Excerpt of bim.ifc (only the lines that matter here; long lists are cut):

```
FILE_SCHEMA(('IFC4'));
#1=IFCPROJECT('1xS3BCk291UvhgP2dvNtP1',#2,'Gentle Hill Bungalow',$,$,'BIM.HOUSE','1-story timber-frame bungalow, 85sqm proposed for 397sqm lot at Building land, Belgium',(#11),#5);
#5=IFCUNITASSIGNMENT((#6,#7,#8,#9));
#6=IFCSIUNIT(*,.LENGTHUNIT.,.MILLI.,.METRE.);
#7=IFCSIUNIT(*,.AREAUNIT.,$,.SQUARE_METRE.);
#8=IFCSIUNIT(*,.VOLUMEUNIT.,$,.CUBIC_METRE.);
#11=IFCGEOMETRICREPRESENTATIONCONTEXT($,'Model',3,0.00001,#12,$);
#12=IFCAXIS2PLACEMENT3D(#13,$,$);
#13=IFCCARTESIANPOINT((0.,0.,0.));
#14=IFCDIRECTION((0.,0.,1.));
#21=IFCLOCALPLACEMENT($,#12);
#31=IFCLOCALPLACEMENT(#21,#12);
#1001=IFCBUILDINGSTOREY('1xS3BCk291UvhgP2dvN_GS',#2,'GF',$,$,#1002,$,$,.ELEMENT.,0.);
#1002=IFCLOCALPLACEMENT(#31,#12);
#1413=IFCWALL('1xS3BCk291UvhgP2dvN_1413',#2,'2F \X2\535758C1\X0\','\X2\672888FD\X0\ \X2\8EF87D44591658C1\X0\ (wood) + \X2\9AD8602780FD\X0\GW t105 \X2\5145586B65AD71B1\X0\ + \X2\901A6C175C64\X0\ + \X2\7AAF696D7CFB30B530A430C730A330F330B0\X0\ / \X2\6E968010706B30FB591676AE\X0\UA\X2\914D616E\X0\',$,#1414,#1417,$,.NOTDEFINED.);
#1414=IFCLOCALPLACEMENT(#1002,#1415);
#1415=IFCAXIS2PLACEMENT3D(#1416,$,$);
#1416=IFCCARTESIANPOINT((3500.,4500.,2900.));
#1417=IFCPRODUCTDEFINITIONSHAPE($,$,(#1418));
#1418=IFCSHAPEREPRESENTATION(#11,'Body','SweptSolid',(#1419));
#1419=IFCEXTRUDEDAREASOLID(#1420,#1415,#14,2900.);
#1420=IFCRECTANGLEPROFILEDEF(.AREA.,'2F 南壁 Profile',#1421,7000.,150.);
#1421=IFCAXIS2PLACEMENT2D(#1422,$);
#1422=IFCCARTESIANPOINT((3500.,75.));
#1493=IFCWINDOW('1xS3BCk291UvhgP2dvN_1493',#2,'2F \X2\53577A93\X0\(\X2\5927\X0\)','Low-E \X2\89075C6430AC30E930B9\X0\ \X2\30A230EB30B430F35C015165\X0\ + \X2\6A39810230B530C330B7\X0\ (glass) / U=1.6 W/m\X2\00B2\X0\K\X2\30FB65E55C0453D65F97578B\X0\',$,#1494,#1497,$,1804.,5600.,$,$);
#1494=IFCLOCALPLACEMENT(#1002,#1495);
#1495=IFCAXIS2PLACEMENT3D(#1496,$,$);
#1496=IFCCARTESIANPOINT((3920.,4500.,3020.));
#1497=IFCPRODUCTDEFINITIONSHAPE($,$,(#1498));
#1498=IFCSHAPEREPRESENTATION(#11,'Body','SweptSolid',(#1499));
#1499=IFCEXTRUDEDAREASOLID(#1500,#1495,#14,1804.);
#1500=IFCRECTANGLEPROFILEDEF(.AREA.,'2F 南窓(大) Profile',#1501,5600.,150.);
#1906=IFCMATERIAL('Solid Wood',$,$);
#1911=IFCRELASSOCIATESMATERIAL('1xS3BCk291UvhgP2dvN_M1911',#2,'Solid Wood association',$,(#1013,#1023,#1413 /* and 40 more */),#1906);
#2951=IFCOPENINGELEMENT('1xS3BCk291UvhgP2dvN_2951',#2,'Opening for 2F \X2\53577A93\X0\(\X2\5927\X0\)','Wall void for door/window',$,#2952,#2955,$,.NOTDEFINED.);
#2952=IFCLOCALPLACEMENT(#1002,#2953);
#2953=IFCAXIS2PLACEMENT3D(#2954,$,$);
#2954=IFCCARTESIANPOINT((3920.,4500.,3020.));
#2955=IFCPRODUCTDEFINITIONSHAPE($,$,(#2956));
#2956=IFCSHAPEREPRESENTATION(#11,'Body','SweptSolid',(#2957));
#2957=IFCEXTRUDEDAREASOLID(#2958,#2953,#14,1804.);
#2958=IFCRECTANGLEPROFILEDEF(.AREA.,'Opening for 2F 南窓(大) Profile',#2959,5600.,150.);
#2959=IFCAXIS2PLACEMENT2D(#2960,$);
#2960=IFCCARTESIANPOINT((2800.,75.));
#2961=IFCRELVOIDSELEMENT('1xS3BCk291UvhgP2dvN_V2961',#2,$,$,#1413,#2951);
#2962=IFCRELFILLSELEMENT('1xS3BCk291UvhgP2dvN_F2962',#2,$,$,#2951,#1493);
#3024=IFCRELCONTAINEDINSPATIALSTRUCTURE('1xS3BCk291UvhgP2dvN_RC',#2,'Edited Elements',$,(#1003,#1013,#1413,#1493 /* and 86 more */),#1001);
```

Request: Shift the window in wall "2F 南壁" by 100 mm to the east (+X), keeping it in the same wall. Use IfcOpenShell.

```python
import ifcopenshell
import ifcopenshell.api.geometry
import ifcopenshell.util.placement
import ifcopenshell.util.unit

model = ifcopenshell.open("bim.ifc")
unit_scale = ifcopenshell.util.unit.calculate_unit_scale(model)

window = model.by_guid("1xS3BCk291UvhgP2dvN_1493")
opening = window.FillsVoids[0].RelatingOpeningElement
wall = opening.VoidsElements[0].RelatingBuildingElement

wall_matrix = ifcopenshell.util.placement.get_local_placement(wall.ObjectPlacement)
shift = wall_matrix[:3, 0] * 0.1 / unit_scale
before = ifcopenshell.util.placement.get_local_placement(window.ObjectPlacement)[:3, 3].copy()

# The window is not placed relative to its opening, so move both.
for product in (opening, window):
    matrix = ifcopenshell.util.placement.get_local_placement(product.ObjectPlacement)
    matrix[:3, 3] += shift
    ifcopenshell.api.geometry.edit_object_placement(model, product=product, matrix=matrix, is_si=False)

after = ifcopenshell.util.placement.get_local_placement(window.ObjectPlacement)[:3, 3]
print("window moved by", (after - before).round(3) + 0.0)

model.write("bim_v2.ifc")
```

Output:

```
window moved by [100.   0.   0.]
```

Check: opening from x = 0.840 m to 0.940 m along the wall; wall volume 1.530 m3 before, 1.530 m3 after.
